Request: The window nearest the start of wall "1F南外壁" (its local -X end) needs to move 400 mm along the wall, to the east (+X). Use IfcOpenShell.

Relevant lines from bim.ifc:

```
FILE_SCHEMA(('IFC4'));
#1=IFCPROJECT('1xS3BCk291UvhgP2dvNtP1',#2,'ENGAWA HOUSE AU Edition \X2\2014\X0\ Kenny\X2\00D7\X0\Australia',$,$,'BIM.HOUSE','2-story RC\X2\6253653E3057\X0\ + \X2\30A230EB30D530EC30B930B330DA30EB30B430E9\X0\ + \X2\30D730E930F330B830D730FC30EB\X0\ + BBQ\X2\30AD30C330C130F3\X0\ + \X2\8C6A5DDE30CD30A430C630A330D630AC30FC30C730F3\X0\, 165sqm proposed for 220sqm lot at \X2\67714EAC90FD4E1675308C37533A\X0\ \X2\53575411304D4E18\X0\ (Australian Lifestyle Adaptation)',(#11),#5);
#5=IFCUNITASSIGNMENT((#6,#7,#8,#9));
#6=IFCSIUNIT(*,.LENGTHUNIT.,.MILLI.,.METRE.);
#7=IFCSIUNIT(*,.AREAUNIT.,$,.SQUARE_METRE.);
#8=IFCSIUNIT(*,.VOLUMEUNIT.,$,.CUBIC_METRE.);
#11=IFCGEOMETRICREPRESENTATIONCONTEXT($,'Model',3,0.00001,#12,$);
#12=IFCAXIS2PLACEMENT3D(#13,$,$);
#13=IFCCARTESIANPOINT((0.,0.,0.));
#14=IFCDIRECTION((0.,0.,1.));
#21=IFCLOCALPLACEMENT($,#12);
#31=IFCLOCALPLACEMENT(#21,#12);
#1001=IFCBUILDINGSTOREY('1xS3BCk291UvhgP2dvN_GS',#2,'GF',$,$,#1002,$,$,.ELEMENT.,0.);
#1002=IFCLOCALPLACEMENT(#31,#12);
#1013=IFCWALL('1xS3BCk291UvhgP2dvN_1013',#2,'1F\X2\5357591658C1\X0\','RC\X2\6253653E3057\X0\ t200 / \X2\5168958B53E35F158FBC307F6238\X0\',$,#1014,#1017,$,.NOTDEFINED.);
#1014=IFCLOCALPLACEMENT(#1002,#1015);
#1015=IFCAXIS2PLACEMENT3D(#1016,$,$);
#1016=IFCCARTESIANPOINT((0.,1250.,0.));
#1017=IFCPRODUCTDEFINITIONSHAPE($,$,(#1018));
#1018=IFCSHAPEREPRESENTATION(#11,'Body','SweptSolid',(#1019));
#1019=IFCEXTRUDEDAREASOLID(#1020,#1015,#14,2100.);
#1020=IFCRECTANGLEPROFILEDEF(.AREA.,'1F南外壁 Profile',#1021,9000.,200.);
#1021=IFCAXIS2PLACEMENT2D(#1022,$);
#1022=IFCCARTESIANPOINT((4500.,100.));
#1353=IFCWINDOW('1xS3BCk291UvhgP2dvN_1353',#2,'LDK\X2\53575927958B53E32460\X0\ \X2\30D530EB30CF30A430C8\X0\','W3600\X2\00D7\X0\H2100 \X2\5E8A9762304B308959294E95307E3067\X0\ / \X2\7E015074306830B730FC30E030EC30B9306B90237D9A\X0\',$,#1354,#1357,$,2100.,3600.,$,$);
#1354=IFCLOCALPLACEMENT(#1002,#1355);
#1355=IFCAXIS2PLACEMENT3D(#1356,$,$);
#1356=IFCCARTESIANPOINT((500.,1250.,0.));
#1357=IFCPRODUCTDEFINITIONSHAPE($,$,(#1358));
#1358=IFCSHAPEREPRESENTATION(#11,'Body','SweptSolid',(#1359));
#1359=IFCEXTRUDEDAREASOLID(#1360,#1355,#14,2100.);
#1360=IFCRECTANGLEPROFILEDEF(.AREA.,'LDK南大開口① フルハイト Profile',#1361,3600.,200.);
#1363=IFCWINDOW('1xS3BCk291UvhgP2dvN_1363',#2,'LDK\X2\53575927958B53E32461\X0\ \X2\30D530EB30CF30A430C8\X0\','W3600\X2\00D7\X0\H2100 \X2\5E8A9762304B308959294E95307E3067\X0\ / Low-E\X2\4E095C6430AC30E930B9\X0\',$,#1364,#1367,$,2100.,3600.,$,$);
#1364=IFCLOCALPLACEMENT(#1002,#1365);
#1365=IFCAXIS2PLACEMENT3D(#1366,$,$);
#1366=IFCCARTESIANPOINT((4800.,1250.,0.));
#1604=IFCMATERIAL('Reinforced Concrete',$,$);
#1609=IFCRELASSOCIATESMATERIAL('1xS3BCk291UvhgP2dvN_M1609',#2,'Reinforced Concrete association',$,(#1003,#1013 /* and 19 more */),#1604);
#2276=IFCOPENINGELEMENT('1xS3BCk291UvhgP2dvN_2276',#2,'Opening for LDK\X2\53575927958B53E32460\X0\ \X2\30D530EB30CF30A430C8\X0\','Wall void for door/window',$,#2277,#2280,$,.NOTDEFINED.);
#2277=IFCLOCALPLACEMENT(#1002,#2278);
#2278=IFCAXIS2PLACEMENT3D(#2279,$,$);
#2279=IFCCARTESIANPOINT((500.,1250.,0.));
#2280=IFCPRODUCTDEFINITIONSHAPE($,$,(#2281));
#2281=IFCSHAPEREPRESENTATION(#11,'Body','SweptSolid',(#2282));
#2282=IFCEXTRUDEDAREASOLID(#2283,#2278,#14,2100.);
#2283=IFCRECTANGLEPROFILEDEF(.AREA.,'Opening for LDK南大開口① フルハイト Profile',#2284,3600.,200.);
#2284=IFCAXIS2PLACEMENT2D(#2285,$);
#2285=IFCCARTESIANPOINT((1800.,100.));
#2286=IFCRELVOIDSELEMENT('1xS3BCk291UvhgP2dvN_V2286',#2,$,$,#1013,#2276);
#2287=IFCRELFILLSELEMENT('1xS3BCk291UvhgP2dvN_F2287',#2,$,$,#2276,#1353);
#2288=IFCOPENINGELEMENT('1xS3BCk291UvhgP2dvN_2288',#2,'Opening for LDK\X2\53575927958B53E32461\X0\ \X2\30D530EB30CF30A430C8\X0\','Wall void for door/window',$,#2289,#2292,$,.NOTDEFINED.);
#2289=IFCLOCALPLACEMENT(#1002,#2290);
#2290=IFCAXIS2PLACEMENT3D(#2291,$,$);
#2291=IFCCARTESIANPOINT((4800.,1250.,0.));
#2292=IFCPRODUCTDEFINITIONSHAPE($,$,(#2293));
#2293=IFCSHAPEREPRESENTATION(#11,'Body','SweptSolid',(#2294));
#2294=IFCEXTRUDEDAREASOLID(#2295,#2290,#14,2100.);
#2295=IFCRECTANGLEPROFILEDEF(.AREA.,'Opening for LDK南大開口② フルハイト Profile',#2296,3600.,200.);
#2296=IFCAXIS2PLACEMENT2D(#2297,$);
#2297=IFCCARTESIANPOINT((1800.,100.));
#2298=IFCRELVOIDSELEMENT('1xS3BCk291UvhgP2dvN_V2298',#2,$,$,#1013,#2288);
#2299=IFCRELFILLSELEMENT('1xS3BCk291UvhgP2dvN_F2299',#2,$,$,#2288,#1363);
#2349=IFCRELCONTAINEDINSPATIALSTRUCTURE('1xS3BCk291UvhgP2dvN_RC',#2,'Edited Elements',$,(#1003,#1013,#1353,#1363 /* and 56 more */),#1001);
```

```python
import ifcopenshell
import ifcopenshell.api.geometry
import ifcopenshell.util.placement

model = ifcopenshell.open("bim.ifc")

window = model.by_id(1353)
opening = window.FillsVoids[0].RelatingOpeningElement
wall = opening.VoidsElements[0].RelatingBuildingElement

wall_matrix = ifcopenshell.util.placement.get_local_placement(wall.ObjectPlacement)
shift = wall_matrix[:3, 0] * 400.0
before = ifcopenshell.util.placement.get_local_placement(window.ObjectPlacement)[:3, 3].copy()

# The window is not placed relative to its opening, so move both.
for product in (opening, window):
    matrix = ifcopenshell.util.placement.get_local_placement(product.ObjectPlacement)
    matrix[:3, 3] += shift
    ifcopenshell.api.geometry.edit_object_placement(model, product=product, matrix=matrix, is_si=False)

after = ifcopenshell.util.placement.get_local_placement(window.ObjectPlacement)[:3, 3]
print("window moved by", (after - before).round(3) + 0.0)

model.write("bim_updated.ifc")
```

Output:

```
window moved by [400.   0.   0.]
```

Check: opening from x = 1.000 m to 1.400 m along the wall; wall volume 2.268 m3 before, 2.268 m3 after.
